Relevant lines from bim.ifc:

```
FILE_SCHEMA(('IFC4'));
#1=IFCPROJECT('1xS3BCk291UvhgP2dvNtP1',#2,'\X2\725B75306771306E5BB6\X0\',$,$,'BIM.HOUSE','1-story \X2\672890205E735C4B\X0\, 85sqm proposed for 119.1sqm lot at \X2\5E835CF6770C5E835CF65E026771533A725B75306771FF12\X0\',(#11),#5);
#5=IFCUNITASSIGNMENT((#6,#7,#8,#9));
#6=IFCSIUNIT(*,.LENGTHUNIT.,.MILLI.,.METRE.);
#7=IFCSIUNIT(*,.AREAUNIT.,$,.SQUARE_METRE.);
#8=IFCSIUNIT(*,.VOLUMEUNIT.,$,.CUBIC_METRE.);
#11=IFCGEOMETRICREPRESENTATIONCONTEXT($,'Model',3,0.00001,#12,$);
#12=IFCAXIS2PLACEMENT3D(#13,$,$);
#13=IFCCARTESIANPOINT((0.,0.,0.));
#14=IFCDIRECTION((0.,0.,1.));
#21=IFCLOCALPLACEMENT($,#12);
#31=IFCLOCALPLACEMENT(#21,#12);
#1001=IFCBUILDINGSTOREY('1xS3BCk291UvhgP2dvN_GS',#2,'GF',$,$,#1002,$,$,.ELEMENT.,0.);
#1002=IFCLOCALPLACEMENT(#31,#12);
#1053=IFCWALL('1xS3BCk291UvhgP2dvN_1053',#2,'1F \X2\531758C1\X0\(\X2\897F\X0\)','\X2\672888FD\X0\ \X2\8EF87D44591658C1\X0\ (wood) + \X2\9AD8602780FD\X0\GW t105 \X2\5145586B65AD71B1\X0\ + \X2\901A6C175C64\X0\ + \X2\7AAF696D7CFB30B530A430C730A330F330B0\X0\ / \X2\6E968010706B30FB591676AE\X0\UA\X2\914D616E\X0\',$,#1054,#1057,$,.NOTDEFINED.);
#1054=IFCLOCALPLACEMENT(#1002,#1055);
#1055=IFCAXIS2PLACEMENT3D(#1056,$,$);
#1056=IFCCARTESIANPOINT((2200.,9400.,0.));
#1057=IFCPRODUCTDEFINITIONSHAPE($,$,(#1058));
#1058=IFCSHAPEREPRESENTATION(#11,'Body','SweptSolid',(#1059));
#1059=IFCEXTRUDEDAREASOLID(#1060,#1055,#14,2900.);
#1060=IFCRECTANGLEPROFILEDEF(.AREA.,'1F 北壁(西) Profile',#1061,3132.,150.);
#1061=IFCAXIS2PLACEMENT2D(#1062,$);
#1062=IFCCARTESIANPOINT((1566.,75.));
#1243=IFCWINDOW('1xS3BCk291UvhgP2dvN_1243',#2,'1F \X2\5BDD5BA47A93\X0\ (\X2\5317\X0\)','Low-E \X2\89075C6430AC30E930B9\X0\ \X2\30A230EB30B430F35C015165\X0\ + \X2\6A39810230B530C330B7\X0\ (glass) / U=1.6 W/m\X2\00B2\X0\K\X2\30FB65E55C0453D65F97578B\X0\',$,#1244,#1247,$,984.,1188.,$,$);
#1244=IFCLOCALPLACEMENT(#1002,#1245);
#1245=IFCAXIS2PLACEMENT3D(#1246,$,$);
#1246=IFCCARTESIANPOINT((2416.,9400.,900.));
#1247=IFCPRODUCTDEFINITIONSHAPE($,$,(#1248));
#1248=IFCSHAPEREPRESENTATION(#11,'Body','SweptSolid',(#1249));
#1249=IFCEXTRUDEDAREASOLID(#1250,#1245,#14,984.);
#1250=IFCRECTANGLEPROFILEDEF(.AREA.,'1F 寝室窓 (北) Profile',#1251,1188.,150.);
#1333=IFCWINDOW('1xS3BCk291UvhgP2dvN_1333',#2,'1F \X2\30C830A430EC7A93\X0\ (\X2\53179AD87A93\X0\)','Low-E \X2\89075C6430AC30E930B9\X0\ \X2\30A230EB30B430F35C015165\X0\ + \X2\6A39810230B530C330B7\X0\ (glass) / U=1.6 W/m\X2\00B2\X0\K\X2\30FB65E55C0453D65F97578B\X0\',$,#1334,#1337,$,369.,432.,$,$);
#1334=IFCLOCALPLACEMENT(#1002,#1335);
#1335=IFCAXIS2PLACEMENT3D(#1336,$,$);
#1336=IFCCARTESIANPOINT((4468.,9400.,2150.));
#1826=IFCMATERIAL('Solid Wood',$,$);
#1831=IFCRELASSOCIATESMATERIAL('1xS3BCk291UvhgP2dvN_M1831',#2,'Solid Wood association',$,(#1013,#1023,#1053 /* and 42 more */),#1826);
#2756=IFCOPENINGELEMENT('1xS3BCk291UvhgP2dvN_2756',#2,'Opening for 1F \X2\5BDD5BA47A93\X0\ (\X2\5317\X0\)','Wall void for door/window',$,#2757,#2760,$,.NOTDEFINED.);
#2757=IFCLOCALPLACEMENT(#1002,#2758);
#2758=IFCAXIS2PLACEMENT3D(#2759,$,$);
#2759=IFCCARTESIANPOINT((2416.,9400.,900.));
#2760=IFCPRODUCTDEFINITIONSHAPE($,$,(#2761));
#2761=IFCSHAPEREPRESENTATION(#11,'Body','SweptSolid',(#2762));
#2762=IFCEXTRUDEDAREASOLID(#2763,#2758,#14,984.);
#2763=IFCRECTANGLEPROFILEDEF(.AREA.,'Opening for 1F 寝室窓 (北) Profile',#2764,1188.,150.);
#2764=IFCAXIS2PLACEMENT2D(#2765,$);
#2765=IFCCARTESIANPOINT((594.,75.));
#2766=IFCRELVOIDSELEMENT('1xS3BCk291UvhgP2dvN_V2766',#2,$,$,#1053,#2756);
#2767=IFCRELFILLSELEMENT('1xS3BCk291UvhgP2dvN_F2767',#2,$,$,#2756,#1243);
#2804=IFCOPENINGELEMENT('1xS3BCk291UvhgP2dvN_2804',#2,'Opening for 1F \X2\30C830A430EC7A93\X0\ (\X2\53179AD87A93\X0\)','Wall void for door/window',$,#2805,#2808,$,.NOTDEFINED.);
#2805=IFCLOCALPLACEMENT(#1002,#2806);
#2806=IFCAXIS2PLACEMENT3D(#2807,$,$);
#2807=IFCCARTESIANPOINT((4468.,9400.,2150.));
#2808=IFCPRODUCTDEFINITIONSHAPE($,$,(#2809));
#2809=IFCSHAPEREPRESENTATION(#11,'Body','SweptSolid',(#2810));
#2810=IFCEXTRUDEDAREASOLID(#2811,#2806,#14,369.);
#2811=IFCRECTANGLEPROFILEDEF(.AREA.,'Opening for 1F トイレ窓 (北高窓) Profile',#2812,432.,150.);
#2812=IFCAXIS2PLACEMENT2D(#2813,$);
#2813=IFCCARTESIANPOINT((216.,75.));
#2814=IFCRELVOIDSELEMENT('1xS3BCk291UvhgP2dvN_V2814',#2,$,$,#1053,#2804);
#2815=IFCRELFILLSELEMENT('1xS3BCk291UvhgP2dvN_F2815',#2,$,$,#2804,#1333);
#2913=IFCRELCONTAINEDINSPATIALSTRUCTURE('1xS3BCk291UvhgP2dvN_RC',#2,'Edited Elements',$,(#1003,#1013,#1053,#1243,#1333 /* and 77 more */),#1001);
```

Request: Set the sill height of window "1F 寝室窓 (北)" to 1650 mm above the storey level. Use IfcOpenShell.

```python
import numpy as np
import ifcopenshell
import ifcopenshell.api.geometry
import ifcopenshell.geom
import ifcopenshell.util.element
import ifcopenshell.util.placement
import ifcopenshell.util.shape
import ifcopenshell.util.unit

model = ifcopenshell.open("bim.ifc")
unit_scale = ifcopenshell.util.unit.calculate_unit_scale(model)

window = model.by_guid("1xS3BCk291UvhgP2dvN_1243")
opening = window.FillsVoids[0].RelatingOpeningElement
storey = ifcopenshell.util.element.get_container(window, ifc_class="IfcBuildingStorey")
level = ifcopenshell.util.placement.get_local_placement(storey.ObjectPlacement)[2, 3]

# The opening's origin need not be at the sill, so measure its lowest point.
shape = ifcopenshell.geom.create_shape(ifcopenshell.geom.settings(), opening)
bottom = ifcopenshell.util.shape.get_shape_bottom_elevation(shape, shape.geometry) / unit_scale
dz = level + 1.65 / unit_scale - bottom

shift = np.array([0.0, 0.0, dz])
# The window is not placed relative to its opening, so move both.
for product in (opening, window):
    matrix = ifcopenshell.util.placement.get_local_placement(product.ObjectPlacement)
    matrix[:3, 3] += shift
    ifcopenshell.api.geometry.edit_object_placement(model, product=product, matrix=matrix, is_si=False)

print(f"moved by {dz * unit_scale:+.3f} m")

model.write("bim_updated.ifc")
```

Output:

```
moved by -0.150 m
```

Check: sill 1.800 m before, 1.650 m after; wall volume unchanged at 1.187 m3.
